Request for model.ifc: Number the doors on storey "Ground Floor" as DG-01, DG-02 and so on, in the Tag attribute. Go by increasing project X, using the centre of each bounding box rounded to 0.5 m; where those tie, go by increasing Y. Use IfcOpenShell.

First a look at what the model holds.

```python
import ifcopenshell
import ifcopenshell.util.element
import ifcopenshell.util.placement

model = ifcopenshell.open("model.ifc")
print(model.schema)
storey = next(s for s in model.by_type("IfcBuildingStorey") if s.Name == "Ground Floor")
doors = [e for e in ifcopenshell.util.element.get_decomposition(storey) if e.is_a("IfcDoor")]
for e in sorted(doors, key=lambda e: e.id()):
    origin = ifcopenshell.util.placement.get_local_placement(e.ObjectPlacement)[:3, 3]
    print(e.id(), e.Tag, e.Name, origin.round(2) + 0.0, sep=" | ")
```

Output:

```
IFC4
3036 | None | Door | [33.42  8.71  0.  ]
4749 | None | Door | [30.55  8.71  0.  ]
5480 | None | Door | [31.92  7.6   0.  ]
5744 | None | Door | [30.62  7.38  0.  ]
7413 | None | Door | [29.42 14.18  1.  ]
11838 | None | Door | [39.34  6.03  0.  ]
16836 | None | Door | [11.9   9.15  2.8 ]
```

```python
import ifcopenshell
import ifcopenshell.geom
import ifcopenshell.util.element
import ifcopenshell.util.shape

model = ifcopenshell.open("model.ifc")
settings = ifcopenshell.geom.settings()
settings.set("use-world-coords", True)


def centre(element):
    shape = ifcopenshell.geom.create_shape(settings, element)
    return ifcopenshell.util.shape.get_bbox_centroid(shape.geometry)


storey = next(s for s in model.by_type("IfcBuildingStorey") if s.Name == "Ground Floor")
doors = [e for e in ifcopenshell.util.element.get_decomposition(storey) if e.is_a("IfcDoor")]

# Insertion points can sit at a corner or the storey origin, so sort by the geometry (in metres).
centres = {e: centre(e) for e in doors}
doors.sort(key=lambda e: (round(centres[e][0] / 0.5), centres[e][1]))

for i, e in enumerate(doors, start=1):
    number = f"DG-{i:02d}"
    e.Tag = number
    print(e.id(), number)

model.write("model_v2.ifc")
```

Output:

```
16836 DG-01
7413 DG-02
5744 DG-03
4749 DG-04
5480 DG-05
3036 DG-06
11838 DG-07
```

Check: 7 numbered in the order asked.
